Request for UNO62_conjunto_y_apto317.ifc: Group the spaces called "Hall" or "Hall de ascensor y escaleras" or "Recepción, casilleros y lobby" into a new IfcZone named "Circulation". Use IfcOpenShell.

First a look at what the model holds.

```python
import ifcopenshell

model = ifcopenshell.open("UNO62_conjunto_y_apto317.ifc")
print(model.schema)
seen = {}
for space in model.by_type("IfcSpace"):
    seen[space.LongName] = seen.get(space.LongName, 0) + 1
for name, count in sorted(seen.items(), key=str):
    print(count, "x", name)
print("zones:", [z.Name for z in model.by_type("IfcZone")][:20])
```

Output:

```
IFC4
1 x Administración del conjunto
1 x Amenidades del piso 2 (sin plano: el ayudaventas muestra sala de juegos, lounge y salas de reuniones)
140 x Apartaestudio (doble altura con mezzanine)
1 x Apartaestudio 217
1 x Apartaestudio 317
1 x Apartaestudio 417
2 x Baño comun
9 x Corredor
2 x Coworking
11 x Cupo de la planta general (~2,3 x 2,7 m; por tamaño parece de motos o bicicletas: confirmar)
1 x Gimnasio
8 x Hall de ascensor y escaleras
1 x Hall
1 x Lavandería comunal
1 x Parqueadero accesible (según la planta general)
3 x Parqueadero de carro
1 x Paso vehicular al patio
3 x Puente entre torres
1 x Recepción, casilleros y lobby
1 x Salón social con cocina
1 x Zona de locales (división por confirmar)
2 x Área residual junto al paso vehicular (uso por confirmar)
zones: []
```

```python
import ifcopenshell
import ifcopenshell.api.group
import ifcopenshell.api.root

model = ifcopenshell.open("UNO62_conjunto_y_apto317.ifc")

names = {"Hall", "Hall de ascensor y escaleras", "Recepción, casilleros y lobby"}
spaces = [s for s in model.by_type("IfcSpace") if s.LongName in names]

zone = ifcopenshell.api.root.create_entity(model, ifc_class="IfcZone", name="Circulation")
ifcopenshell.api.group.assign_group(model, products=spaces, group=zone)
print(len(spaces), "spaces in", zone.Name)

model.write("UNO62_conjunto_y_apto317-out.ifc")
```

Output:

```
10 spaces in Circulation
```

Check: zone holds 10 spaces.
